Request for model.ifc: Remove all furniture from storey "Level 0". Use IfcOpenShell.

First a look at what the model holds.

```python
import ifcopenshell
import ifcopenshell.util.element

model = ifcopenshell.open("model.ifc")
print(model.schema)
storey = next(s for s in model.by_type("IfcBuildingStorey") if s.Name == "Level 0")
furniture = [e for e in ifcopenshell.util.element.get_decomposition(storey) if e.is_a("IfcFurnishingElement")]
seen = {}
for e in furniture:
    element_type = ifcopenshell.util.element.get_type(e)
    name = element_type.Name if element_type not in (None, e) else None
    seen[name] = seen.get(name, 0) + 1
for name, count in sorted(seen.items(), key=str):
    print(count, "x", name)
```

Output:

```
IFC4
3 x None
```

```python
import ifcopenshell
import ifcopenshell.api.root
import ifcopenshell.util.element

model = ifcopenshell.open("model.ifc")

storey = next(s for s in model.by_type("IfcBuildingStorey") if s.Name == "Level 0")
furniture = [e for e in ifcopenshell.util.element.get_decomposition(storey) if e.is_a("IfcFurnishingElement")]

for e in furniture:
    ifcopenshell.api.root.remove_product(model, product=e)
print(len(furniture), "removed")

model.write("model_v2.ifc")
```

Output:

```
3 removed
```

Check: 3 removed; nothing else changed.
